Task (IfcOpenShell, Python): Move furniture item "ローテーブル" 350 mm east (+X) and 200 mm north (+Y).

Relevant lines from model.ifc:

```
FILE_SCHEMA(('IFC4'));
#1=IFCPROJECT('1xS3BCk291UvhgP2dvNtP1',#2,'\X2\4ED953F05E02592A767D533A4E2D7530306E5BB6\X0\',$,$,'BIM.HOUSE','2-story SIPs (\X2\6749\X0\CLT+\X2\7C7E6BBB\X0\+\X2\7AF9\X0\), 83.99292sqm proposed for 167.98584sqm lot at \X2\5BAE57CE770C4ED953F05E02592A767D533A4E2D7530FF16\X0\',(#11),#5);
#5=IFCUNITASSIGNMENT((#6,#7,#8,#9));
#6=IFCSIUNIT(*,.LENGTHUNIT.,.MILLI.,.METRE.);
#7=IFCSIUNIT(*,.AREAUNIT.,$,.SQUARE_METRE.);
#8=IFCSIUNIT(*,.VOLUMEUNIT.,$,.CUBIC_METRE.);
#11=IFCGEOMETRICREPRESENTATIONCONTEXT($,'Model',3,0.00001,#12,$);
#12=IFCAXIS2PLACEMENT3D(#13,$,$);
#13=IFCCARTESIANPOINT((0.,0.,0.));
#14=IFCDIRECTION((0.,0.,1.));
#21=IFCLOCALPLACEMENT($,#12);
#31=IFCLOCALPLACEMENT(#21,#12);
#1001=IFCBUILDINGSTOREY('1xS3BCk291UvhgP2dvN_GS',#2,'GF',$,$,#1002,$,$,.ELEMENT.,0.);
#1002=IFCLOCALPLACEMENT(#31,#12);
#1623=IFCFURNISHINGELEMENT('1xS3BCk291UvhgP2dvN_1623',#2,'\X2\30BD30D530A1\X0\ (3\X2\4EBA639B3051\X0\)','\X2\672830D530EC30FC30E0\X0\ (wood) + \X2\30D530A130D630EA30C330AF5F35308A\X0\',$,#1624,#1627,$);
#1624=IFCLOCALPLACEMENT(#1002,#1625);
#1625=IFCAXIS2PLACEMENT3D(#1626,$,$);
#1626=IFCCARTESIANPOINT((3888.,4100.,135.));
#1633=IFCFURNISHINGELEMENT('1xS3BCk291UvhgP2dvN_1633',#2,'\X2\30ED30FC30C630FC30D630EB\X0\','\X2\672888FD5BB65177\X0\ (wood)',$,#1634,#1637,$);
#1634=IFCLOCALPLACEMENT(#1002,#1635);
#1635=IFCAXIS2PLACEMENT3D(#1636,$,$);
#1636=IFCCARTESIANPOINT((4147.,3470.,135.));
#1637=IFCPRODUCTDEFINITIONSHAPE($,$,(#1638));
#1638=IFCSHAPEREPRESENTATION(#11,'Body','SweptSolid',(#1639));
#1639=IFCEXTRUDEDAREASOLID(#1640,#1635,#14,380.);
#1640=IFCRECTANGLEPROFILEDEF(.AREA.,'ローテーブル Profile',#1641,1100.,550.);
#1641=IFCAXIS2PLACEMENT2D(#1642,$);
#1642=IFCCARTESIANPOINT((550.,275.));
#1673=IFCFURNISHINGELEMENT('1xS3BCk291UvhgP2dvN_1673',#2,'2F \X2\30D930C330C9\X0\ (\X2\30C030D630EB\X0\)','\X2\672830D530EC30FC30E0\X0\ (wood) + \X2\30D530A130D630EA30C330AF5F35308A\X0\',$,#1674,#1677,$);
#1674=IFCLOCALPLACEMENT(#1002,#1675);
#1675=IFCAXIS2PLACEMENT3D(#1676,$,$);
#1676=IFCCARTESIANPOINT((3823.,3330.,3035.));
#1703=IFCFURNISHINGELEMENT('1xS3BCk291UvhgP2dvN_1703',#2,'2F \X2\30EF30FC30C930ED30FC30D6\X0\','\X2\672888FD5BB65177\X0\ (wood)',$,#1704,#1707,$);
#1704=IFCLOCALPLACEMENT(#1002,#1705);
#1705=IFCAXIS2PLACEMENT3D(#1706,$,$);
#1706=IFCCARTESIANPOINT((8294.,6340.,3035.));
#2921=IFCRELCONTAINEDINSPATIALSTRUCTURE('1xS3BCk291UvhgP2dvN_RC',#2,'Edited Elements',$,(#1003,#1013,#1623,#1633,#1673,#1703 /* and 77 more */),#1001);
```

```python
import ifcopenshell
import ifcopenshell.api.geometry
import ifcopenshell.util.placement

model = ifcopenshell.open("model.ifc")

item = model.by_id(1633)
matrix = ifcopenshell.util.placement.get_local_placement(item.ObjectPlacement)
matrix[0, 3] += 350.0
matrix[1, 3] += 200.0
ifcopenshell.api.geometry.edit_object_placement(model, product=item, matrix=matrix, is_si=False)

print(ifcopenshell.util.placement.get_local_placement(item.ObjectPlacement).round(3) + 0.0)

model.write("model_v2.ifc")
```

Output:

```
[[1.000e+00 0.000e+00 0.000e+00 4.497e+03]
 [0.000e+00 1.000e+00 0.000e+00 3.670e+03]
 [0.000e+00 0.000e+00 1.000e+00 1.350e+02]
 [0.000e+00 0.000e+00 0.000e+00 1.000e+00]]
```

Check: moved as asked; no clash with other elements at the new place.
